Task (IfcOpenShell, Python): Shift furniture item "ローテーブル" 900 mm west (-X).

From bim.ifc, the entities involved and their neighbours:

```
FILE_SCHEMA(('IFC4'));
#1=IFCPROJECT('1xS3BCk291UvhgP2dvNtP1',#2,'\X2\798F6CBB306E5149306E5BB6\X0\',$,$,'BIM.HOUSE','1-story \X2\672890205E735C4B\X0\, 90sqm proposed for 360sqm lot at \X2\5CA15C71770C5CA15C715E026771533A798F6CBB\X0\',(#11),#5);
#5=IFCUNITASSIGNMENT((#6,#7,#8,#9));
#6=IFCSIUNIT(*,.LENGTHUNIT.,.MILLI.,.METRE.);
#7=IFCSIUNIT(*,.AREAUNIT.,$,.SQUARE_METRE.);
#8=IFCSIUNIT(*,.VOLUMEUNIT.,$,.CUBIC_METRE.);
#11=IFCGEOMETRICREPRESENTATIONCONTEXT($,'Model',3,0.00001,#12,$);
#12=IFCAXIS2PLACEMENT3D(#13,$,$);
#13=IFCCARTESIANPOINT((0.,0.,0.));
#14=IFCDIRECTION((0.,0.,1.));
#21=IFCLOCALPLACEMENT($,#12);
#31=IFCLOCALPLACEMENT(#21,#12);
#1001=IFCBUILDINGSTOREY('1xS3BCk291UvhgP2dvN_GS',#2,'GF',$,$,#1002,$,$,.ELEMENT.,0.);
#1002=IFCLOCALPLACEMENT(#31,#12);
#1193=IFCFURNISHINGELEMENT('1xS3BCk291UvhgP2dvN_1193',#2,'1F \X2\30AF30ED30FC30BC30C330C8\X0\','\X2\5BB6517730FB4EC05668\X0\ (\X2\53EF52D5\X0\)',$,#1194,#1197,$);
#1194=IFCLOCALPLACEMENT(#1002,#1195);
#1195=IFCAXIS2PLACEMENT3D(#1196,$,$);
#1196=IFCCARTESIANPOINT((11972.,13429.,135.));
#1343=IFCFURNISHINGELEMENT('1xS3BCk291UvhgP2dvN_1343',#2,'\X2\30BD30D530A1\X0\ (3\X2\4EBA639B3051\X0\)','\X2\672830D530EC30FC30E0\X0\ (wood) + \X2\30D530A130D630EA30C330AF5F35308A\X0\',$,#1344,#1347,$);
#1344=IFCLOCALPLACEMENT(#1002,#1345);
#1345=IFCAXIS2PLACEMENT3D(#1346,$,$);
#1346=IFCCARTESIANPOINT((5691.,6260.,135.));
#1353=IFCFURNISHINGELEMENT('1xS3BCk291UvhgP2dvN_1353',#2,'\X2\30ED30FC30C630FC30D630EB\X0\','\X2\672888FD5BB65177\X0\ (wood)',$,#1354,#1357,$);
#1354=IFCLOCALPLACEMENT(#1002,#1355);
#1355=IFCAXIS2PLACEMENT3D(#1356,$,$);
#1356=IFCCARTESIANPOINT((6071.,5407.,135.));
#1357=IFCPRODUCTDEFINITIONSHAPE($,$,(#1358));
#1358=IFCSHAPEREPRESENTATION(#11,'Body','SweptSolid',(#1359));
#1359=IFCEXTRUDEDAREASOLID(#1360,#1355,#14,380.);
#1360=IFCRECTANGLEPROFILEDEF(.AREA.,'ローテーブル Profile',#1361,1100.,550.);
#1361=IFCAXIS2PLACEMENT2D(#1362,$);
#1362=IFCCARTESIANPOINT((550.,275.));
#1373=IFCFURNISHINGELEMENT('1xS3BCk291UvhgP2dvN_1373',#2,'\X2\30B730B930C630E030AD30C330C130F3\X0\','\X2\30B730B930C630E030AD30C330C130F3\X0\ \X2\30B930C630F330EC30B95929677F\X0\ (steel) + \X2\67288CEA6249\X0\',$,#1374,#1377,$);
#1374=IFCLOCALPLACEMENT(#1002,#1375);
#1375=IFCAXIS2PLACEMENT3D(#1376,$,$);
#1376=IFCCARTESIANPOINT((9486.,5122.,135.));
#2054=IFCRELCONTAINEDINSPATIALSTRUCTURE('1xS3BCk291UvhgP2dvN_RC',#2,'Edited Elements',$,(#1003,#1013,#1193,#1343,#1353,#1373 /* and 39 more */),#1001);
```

```python
import ifcopenshell
import ifcopenshell.api.geometry
import ifcopenshell.util.placement

model = ifcopenshell.open("bim.ifc")

item = model.by_guid("1xS3BCk291UvhgP2dvN_1353")
matrix = ifcopenshell.util.placement.get_local_placement(item.ObjectPlacement)
matrix[0, 3] -= 900.0
ifcopenshell.api.geometry.edit_object_placement(model, product=item, matrix=matrix, is_si=False)

print(ifcopenshell.util.placement.get_local_placement(item.ObjectPlacement).round(3) + 0.0)

model.write("bim_updated.ifc")
```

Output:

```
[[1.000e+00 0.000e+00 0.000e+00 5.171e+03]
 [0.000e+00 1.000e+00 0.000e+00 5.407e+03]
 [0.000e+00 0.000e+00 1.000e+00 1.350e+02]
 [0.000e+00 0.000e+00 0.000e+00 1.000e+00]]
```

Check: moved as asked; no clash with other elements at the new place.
